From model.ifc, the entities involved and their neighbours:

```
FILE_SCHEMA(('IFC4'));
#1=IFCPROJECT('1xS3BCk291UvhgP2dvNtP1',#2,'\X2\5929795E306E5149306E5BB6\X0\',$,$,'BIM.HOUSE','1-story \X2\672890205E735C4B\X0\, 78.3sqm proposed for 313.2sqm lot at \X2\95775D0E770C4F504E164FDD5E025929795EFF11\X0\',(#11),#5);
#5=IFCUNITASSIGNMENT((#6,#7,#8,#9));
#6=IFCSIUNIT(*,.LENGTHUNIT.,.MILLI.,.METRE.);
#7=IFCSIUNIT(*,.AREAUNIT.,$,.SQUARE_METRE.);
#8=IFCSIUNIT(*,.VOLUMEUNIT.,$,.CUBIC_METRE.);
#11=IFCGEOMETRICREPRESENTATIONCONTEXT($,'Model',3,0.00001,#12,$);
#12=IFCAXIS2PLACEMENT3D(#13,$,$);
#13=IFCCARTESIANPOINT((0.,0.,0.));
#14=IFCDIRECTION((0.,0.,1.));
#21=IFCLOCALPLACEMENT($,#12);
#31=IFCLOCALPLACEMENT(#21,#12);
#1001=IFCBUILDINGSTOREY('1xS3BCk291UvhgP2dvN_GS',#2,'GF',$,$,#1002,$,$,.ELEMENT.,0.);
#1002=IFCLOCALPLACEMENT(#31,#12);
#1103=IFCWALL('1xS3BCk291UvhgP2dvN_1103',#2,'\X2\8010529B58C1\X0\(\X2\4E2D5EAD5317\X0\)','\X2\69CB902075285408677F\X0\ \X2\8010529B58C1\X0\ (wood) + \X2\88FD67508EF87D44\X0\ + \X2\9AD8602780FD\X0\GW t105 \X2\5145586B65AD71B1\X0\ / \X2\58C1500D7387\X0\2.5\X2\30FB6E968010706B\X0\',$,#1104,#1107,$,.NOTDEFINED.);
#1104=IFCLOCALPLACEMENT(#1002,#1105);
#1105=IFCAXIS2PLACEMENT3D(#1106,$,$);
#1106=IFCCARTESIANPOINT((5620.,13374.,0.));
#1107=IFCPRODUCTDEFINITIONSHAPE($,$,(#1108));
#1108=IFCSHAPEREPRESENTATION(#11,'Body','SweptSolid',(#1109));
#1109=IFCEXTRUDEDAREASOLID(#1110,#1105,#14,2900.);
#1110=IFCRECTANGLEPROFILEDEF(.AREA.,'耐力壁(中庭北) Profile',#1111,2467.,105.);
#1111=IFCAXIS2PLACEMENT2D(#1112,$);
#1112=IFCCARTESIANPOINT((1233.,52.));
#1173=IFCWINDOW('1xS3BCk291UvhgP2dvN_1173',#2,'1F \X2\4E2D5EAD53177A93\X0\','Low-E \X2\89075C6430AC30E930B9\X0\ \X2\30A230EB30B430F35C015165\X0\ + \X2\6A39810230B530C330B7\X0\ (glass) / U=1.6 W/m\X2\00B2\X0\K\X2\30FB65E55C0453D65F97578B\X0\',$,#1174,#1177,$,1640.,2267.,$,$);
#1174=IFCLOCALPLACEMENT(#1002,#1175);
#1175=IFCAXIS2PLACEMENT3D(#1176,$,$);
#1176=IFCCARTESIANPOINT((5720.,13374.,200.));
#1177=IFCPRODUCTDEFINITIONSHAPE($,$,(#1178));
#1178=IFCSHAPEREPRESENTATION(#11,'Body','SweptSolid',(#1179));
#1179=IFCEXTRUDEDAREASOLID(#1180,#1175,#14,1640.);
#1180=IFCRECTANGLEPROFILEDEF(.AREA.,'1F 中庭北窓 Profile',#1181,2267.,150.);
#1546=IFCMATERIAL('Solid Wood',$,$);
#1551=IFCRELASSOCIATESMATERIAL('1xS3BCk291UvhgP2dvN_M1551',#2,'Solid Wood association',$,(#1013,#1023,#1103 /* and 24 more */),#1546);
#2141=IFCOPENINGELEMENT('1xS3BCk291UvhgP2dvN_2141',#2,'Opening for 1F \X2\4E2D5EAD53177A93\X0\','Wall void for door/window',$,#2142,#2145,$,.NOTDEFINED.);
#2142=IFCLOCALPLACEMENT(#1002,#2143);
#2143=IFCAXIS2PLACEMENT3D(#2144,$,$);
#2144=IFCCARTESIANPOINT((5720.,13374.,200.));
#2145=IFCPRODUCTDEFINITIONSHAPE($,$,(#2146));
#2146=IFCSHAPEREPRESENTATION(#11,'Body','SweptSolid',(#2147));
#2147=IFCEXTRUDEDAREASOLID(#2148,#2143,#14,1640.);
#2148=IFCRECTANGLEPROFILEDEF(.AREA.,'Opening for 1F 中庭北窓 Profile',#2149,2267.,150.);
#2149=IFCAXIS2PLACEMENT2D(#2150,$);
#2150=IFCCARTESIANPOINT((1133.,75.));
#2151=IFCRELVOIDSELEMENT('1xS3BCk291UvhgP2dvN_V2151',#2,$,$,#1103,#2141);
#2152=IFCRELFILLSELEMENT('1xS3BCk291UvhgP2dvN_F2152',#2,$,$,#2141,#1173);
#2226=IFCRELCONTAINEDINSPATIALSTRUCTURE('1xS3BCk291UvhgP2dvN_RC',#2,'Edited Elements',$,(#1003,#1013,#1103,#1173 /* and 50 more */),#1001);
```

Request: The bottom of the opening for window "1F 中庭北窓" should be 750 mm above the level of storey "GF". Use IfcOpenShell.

```python
import numpy as np
import ifcopenshell
import ifcopenshell.api.geometry
import ifcopenshell.geom
import ifcopenshell.util.element
import ifcopenshell.util.placement
import ifcopenshell.util.shape
import ifcopenshell.util.unit

model = ifcopenshell.open("model.ifc")
unit_scale = ifcopenshell.util.unit.calculate_unit_scale(model)

window = model.by_guid("1xS3BCk291UvhgP2dvN_1173")
opening = window.FillsVoids[0].RelatingOpeningElement
storey = ifcopenshell.util.element.get_container(window, ifc_class="IfcBuildingStorey")
level = ifcopenshell.util.placement.get_local_placement(storey.ObjectPlacement)[2, 3]

# The opening's origin need not be at the sill, so measure its lowest point.
shape = ifcopenshell.geom.create_shape(ifcopenshell.geom.settings(), opening)
bottom = ifcopenshell.util.shape.get_shape_bottom_elevation(shape, shape.geometry) / unit_scale
dz = level + 750.0 - bottom

shift = np.array([0.0, 0.0, dz])
# The window is not placed relative to its opening, so move both.
for product in (opening, window):
    matrix = ifcopenshell.util.placement.get_local_placement(product.ObjectPlacement)
    matrix[:3, 3] += shift
    ifcopenshell.api.geometry.edit_object_placement(model, product=product, matrix=matrix, is_si=False)

print(f"moved by {dz * unit_scale:+.3f} m")

model.write("model_edited.ifc")
```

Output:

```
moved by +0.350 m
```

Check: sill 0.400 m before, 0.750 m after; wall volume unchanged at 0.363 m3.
